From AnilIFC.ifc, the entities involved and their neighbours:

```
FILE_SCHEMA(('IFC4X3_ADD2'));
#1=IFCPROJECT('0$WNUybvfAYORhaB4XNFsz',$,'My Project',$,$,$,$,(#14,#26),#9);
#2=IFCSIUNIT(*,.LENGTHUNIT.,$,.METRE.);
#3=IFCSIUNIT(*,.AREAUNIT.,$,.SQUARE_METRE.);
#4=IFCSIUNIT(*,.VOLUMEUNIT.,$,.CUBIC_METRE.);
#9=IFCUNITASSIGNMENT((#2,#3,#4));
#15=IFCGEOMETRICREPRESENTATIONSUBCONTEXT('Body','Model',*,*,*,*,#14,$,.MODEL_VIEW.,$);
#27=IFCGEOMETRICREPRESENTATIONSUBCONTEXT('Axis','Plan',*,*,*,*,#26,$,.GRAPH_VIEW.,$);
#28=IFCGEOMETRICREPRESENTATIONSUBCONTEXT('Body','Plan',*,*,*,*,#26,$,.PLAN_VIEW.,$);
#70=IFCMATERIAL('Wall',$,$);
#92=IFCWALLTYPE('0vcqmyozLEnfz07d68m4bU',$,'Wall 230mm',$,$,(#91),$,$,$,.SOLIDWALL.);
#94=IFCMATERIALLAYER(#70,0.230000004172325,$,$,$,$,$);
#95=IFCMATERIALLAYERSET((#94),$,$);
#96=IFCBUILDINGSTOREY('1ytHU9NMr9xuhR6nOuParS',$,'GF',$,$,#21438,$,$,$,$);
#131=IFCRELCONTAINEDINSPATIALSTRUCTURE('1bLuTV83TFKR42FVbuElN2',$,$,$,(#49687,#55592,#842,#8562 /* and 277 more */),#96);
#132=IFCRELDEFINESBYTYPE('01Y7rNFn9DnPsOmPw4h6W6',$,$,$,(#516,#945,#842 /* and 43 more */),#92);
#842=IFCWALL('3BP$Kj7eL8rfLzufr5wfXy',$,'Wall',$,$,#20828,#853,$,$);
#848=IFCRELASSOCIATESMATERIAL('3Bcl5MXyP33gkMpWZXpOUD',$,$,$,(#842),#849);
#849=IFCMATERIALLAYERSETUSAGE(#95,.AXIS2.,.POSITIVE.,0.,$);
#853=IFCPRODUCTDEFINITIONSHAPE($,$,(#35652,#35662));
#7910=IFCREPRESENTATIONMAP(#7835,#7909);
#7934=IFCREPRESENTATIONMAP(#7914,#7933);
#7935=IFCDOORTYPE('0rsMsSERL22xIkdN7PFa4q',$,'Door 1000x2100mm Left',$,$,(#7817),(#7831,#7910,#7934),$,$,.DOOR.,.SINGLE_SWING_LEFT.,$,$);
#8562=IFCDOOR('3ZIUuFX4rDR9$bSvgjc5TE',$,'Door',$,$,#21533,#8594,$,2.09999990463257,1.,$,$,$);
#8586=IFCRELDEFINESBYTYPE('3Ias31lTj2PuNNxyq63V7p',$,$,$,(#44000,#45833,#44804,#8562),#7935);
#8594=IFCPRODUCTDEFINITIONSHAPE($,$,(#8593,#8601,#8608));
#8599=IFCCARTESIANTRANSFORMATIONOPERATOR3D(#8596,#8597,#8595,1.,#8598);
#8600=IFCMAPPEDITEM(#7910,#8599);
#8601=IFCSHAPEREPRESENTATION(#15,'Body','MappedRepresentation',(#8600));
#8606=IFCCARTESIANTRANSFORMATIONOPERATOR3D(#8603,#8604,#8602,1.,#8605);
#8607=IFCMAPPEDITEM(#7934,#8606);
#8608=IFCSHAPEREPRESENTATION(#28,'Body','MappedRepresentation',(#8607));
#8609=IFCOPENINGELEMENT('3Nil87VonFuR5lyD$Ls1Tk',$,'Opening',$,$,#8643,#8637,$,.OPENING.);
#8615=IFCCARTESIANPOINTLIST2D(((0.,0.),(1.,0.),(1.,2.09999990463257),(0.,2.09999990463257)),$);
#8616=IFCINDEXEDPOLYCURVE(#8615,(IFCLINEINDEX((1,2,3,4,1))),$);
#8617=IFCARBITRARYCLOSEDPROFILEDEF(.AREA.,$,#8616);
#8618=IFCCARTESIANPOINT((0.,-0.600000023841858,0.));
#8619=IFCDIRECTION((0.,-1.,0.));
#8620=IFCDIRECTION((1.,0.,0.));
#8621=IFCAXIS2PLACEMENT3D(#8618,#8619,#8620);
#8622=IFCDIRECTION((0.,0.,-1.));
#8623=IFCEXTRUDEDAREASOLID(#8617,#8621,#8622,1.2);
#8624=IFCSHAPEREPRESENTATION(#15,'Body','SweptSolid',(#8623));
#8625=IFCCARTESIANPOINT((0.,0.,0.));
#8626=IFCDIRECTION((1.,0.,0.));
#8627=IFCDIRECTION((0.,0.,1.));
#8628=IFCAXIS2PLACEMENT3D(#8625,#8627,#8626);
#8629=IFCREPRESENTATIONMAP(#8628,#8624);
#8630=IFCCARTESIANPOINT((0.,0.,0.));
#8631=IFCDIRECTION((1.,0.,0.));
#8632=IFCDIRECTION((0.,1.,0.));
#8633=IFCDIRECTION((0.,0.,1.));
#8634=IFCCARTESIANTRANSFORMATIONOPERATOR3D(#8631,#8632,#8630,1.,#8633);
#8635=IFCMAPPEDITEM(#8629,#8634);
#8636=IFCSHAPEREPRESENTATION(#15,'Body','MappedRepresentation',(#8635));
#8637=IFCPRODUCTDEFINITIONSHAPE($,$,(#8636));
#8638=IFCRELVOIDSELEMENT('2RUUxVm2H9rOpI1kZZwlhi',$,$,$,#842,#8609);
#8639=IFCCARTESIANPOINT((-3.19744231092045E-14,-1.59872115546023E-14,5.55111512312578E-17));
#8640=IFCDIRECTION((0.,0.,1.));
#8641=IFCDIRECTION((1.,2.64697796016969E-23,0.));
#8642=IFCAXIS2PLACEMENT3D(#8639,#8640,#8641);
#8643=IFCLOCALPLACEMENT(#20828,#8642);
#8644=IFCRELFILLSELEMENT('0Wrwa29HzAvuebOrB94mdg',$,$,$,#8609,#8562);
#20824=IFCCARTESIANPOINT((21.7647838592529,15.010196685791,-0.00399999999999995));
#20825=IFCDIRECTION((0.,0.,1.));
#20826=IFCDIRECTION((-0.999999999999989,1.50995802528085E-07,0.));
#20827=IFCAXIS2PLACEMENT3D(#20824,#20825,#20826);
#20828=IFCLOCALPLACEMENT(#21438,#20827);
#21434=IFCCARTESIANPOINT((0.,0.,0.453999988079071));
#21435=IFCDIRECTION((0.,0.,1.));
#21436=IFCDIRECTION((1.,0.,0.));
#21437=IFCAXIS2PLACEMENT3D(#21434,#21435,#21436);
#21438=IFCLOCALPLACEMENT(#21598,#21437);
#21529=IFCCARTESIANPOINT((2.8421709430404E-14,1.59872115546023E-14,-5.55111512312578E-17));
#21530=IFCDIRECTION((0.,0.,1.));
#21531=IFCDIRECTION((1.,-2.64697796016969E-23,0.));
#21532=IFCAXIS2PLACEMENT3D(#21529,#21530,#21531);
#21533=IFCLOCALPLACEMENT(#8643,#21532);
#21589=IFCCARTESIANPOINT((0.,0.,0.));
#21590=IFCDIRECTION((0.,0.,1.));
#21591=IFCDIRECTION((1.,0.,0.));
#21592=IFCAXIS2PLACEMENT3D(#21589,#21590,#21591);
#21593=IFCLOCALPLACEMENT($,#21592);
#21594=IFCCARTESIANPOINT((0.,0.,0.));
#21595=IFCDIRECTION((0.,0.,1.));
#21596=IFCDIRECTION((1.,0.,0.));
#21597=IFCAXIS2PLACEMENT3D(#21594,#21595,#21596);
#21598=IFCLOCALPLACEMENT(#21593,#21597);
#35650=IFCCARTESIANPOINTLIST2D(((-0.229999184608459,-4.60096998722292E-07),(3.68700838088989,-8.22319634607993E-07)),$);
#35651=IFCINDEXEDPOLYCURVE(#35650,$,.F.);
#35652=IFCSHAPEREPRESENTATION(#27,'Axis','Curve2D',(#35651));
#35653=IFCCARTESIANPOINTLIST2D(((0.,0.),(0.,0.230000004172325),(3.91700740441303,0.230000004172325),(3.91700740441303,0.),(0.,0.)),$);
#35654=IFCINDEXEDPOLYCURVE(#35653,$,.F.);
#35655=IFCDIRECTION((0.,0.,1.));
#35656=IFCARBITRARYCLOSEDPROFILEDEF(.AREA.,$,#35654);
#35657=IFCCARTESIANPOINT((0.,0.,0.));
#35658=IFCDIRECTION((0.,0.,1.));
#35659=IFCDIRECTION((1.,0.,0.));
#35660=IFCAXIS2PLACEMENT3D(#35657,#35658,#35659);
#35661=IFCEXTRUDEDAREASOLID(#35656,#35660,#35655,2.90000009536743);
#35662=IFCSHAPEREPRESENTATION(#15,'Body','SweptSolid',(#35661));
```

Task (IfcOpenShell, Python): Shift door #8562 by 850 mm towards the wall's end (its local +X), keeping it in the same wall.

```python
import ifcopenshell
import ifcopenshell.api.geometry
import ifcopenshell.util.placement

model = ifcopenshell.open("AnilIFC.ifc")

door = model.by_guid("3ZIUuFX4rDR9$bSvgjc5TE")
opening = door.FillsVoids[0].RelatingOpeningElement
wall = opening.VoidsElements[0].RelatingBuildingElement

wall_matrix = ifcopenshell.util.placement.get_local_placement(wall.ObjectPlacement)
shift = wall_matrix[:3, 0] * 0.85
before = ifcopenshell.util.placement.get_local_placement(door.ObjectPlacement)[:3, 3].copy()

# The door is placed relative to its opening, so it follows when the opening moves.
matrix = ifcopenshell.util.placement.get_local_placement(opening.ObjectPlacement)
matrix[:3, 3] += shift
ifcopenshell.api.geometry.edit_object_placement(
    model, product=opening, matrix=matrix, is_si=False, should_transform_children=True
)

after = ifcopenshell.util.placement.get_local_placement(door.ObjectPlacement)[:3, 3]
print("door moved by", (after - before).round(3) + 0.0)

model.write("AnilIFC_v2.ifc")
```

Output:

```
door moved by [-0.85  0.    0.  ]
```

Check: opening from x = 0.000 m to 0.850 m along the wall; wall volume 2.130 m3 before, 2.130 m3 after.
